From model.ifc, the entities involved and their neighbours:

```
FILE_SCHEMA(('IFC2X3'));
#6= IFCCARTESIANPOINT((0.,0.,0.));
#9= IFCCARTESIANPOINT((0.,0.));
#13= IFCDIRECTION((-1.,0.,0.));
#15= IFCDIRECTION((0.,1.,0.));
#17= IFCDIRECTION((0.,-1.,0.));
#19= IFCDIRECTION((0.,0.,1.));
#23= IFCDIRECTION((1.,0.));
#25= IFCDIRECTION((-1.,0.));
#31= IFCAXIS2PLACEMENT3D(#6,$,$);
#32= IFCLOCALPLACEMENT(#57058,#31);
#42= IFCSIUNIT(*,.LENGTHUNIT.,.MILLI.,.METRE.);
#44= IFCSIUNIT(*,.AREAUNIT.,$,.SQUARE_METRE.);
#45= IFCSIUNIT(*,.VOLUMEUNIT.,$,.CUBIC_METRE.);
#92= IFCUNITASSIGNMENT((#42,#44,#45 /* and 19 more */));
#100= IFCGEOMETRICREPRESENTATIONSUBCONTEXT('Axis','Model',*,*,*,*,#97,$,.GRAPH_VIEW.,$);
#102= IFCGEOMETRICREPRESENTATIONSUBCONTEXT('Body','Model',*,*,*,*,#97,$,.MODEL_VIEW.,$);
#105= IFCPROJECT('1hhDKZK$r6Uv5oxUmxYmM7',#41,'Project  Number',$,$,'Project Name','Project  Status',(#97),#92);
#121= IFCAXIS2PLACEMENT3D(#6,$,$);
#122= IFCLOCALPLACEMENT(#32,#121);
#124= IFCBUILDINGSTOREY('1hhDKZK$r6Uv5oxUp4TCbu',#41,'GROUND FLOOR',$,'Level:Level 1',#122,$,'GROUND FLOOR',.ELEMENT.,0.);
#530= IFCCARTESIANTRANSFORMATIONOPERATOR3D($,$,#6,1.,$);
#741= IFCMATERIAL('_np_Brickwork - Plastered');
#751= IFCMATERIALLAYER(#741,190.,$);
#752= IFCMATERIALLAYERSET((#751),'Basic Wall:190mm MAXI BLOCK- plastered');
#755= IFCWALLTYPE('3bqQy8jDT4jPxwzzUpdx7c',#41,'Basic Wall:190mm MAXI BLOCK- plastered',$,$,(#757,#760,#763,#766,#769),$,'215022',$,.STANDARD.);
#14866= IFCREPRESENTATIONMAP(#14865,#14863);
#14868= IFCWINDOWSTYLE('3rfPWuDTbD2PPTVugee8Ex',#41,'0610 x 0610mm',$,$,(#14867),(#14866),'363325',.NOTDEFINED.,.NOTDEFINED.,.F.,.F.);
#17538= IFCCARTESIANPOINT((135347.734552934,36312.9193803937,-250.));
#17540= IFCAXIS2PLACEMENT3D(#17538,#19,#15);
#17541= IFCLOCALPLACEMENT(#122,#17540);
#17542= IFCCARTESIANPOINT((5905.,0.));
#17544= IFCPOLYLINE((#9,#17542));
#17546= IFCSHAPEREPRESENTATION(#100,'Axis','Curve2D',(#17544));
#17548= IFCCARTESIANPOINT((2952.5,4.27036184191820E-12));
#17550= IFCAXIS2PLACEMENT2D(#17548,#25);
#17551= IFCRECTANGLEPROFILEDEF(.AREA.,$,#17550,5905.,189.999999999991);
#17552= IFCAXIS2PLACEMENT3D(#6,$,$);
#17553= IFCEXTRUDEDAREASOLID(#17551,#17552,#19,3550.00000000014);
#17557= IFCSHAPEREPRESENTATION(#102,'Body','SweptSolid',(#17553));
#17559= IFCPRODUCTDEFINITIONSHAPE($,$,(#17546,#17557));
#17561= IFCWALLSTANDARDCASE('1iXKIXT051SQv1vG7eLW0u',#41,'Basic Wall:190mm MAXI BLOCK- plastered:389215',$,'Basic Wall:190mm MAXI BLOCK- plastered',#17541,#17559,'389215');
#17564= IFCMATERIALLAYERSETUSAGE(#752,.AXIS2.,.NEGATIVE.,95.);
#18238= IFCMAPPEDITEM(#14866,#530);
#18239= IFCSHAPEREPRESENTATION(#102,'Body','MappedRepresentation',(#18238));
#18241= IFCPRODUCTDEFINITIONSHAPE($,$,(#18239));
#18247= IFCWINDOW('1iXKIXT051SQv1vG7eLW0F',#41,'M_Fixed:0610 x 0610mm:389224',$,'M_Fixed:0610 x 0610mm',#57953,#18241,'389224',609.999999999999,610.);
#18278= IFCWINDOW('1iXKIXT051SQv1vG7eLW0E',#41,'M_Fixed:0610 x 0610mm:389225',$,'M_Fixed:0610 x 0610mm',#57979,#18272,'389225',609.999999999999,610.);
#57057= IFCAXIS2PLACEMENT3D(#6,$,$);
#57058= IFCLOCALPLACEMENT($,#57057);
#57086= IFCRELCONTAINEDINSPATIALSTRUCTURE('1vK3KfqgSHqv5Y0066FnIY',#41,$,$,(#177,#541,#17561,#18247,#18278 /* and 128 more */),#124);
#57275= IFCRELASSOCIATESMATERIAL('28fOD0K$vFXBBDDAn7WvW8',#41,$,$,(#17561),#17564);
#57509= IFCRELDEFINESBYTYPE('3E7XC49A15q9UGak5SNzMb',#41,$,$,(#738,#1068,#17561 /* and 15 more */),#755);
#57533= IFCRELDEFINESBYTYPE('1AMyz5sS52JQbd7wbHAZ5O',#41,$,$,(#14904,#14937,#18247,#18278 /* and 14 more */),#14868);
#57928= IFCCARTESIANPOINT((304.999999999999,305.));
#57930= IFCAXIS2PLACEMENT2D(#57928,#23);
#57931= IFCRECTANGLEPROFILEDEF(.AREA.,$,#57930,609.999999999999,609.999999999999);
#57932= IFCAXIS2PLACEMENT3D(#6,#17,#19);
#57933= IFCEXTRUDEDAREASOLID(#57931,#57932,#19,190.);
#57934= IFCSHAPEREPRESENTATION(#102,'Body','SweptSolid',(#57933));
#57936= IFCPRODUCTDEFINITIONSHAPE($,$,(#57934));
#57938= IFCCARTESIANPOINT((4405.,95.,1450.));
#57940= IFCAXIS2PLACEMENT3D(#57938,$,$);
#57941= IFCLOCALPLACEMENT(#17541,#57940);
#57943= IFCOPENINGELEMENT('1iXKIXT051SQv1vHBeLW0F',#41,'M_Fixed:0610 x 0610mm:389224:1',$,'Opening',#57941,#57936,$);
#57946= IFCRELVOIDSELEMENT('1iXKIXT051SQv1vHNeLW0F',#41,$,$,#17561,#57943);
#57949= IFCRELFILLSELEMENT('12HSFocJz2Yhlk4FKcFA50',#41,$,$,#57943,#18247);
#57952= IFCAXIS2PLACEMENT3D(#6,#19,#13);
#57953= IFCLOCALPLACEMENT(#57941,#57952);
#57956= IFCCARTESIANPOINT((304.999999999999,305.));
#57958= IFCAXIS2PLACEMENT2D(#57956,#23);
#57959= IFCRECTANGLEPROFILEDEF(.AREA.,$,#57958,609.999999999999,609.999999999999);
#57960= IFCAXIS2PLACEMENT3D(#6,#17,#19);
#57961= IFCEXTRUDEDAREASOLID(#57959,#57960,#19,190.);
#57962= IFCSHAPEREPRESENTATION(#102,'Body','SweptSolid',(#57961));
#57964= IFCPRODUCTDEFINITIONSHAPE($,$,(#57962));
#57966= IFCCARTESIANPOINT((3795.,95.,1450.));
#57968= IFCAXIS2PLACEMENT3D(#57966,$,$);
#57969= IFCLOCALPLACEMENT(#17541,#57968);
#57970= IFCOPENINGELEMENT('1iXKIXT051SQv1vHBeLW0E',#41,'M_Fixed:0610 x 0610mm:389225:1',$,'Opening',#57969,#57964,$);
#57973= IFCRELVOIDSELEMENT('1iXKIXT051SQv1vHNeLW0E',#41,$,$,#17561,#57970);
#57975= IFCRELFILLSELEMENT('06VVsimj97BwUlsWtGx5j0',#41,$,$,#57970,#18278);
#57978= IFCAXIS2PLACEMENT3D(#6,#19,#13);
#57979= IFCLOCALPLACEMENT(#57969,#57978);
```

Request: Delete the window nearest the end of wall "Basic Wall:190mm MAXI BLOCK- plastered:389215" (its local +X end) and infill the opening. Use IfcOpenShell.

```python
import ifcopenshell
import ifcopenshell.api.feature
import ifcopenshell.api.root
import ifcopenshell.geom
import ifcopenshell.util.shape

model = ifcopenshell.open("model.ifc")
settings = ifcopenshell.geom.settings()


def volume(element):
    """Net volume in cubic metres, openings subtracted."""
    shape = ifcopenshell.geom.create_shape(settings, element)
    return ifcopenshell.util.shape.get_volume(shape.geometry)


window = model.by_guid("1iXKIXT051SQv1vG7eLW0F")
opening = window.FillsVoids[0].RelatingOpeningElement
wall = opening.VoidsElements[0].RelatingBuildingElement
before = volume(wall)

ifcopenshell.api.root.remove_product(model, product=window)
ifcopenshell.api.feature.remove_feature(model, feature=opening)

after = volume(wall)

print(f"wall volume {before:.3f} -> {after:.3f} m3")

model.write("model-out.ifc")
```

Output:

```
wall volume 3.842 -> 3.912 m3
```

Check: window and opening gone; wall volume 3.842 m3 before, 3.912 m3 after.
